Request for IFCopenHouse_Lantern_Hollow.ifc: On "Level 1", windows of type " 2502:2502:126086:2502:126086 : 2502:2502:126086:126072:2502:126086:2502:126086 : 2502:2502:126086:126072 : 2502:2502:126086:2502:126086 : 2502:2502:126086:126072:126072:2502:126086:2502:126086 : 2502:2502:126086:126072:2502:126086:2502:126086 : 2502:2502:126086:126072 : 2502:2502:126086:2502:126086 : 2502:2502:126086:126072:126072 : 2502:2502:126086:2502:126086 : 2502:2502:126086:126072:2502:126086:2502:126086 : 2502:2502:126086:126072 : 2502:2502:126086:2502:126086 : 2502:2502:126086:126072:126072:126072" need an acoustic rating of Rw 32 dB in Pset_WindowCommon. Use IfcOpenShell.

First a look at what the model holds.

```python
import ifcopenshell
import ifcopenshell.util.element

model = ifcopenshell.open("IFCopenHouse_Lantern_Hollow.ifc")
print(model.schema)
storey = next(s for s in model.by_type("IfcBuildingStorey") if s.Name == "Level 1")
windows = [e for e in ifcopenshell.util.element.get_decomposition(storey) if e.is_a("IfcWindow")]
seen = {}
for e in windows:
    element_type = ifcopenshell.util.element.get_type(e)
    key = (element_type.Name if element_type != e and element_type else None, ifcopenshell.util.element.get_pset(e, "Pset_WindowCommon", "AcousticRating"))
    seen[key] = seen.get(key, 0) + 1
for (name, value), count in sorted(seen.items(), key=str):
    print(count, "x", name, "|", value)
```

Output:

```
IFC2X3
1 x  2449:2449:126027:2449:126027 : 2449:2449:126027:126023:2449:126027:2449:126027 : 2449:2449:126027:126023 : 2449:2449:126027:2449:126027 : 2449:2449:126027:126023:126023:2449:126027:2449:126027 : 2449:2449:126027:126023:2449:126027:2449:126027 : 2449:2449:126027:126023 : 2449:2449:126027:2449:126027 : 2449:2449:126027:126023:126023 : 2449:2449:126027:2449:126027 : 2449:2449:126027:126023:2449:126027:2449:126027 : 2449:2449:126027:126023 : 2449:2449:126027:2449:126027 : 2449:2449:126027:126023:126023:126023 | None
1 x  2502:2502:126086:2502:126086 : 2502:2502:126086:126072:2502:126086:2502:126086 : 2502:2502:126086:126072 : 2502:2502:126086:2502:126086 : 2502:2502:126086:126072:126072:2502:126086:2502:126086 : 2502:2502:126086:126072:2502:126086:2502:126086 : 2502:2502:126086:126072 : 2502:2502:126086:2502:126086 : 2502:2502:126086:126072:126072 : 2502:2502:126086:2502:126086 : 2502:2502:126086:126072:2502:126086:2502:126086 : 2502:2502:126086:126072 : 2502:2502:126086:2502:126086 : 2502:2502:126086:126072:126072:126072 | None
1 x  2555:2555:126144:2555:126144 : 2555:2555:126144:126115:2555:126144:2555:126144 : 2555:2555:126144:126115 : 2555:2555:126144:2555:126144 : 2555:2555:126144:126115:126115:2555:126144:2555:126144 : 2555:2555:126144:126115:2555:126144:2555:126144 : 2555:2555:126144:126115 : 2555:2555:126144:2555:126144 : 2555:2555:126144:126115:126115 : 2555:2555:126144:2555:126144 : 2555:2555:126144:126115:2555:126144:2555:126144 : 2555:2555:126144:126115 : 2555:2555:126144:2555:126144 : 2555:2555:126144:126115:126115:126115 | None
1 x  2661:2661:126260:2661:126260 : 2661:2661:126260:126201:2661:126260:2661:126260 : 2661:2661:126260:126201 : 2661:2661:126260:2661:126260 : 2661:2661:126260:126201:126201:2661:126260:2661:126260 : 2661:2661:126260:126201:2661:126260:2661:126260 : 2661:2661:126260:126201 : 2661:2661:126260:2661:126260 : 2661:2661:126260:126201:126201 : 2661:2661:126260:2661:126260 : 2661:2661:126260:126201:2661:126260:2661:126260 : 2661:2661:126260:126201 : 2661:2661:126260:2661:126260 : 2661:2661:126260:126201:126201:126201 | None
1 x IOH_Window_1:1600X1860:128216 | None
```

```python
import ifcopenshell
import ifcopenshell.api.pset
import ifcopenshell.util.element

model = ifcopenshell.open("IFCopenHouse_Lantern_Hollow.ifc")

storey = next(s for s in model.by_type("IfcBuildingStorey") if s.Name == "Level 1")
windows = [e for e in ifcopenshell.util.element.get_decomposition(storey) if e.is_a("IfcWindow")]

count = 0
for e in windows:
    element_type = ifcopenshell.util.element.get_type(e)
    if element_type in (None, e) or element_type.Name != " 2502:2502:126086:2502:126086 : 2502:2502:126086:126072:2502:126086:2502:126086 : 2502:2502:126086:126072 : 2502:2502:126086:2502:126086 : 2502:2502:126086:126072:126072:2502:126086:2502:126086 : 2502:2502:126086:126072:2502:126086:2502:126086 : 2502:2502:126086:126072 : 2502:2502:126086:2502:126086 : 2502:2502:126086:126072:126072 : 2502:2502:126086:2502:126086 : 2502:2502:126086:126072:2502:126086:2502:126086 : 2502:2502:126086:126072 : 2502:2502:126086:2502:126086 : 2502:2502:126086:126072:126072:126072":
        continue
    # add_pset returns the element's existing set when there is one.
    pset = ifcopenshell.api.pset.add_pset(model, product=e, name="Pset_WindowCommon")
    ifcopenshell.api.pset.edit_pset(model, pset=pset, properties={"AcousticRating": "Rw 32 dB"})
    count += 1

print(count, "windows updated")

model.write("IFCopenHouse_Lantern_Hollow_updated.ifc")
```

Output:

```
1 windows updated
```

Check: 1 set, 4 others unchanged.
